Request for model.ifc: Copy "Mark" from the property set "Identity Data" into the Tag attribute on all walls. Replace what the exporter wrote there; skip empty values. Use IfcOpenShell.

First a look at what the model holds.

```python
import ifcopenshell
import ifcopenshell.util.element

model = ifcopenshell.open("model.ifc")
print(model.schema)
walls = model.by_type("IfcWall")
print(len(walls), "walls")
for e in walls[:8]:
    source = ifcopenshell.util.element.get_pset(e, "Identity Data", "Mark")
    target = e.Tag
    print(e.id(), repr(source), repr(target), sep=" | ")
```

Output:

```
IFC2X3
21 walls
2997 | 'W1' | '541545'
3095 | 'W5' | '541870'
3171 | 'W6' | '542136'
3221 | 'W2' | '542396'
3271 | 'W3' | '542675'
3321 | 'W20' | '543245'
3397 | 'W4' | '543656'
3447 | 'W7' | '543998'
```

```python
import ifcopenshell
import ifcopenshell.util.element

model = ifcopenshell.open("model.ifc")

count = 0
for e in model.by_type("IfcWall"):
    value = ifcopenshell.util.element.get_pset(e, "Identity Data", "Mark")
    current = e.Tag
    if not value or not value.strip() or current == value:
        continue
    e.Tag = value
    count += 1

print(count, "walls updated")

model.write("model_rev.ifc")
```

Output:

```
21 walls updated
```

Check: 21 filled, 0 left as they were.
